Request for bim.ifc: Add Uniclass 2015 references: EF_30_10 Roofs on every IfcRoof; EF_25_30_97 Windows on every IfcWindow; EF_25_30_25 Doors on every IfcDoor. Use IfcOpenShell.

First a look at what the model holds.

```python
import ifcopenshell

model = ifcopenshell.open("bim.ifc")
print(model.schema)
print("classifications:", [c.Name for c in model.by_type("IfcClassification")])
for ifc_class in ("IfcDoor", "IfcRoof", "IfcStair", "IfcWall", "IfcWindow"):
    print(ifc_class, len(model.by_type(ifc_class)))
```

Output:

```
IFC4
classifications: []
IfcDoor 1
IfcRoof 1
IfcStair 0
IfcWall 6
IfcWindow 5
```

```python
import ifcopenshell
import ifcopenshell.api.classification

model = ifcopenshell.open("bim.ifc")

system = ifcopenshell.api.classification.add_classification(model, classification="Uniclass 2015")

codes = {
    "IfcRoof": ("EF_30_10", "Roofs"),
    "IfcWindow": ("EF_25_30_97", "Windows"),
    "IfcDoor": ("EF_25_30_25", "Doors"),
}
for ifc_class, (code, name) in codes.items():
    products = model.by_type(ifc_class)
    ifcopenshell.api.classification.add_reference(
        model, products=products, classification=system, identification=code, name=name
    )
    print(code, len(products))

model.write("bim-out.ifc")
```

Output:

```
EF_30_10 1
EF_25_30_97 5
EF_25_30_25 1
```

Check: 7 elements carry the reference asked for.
